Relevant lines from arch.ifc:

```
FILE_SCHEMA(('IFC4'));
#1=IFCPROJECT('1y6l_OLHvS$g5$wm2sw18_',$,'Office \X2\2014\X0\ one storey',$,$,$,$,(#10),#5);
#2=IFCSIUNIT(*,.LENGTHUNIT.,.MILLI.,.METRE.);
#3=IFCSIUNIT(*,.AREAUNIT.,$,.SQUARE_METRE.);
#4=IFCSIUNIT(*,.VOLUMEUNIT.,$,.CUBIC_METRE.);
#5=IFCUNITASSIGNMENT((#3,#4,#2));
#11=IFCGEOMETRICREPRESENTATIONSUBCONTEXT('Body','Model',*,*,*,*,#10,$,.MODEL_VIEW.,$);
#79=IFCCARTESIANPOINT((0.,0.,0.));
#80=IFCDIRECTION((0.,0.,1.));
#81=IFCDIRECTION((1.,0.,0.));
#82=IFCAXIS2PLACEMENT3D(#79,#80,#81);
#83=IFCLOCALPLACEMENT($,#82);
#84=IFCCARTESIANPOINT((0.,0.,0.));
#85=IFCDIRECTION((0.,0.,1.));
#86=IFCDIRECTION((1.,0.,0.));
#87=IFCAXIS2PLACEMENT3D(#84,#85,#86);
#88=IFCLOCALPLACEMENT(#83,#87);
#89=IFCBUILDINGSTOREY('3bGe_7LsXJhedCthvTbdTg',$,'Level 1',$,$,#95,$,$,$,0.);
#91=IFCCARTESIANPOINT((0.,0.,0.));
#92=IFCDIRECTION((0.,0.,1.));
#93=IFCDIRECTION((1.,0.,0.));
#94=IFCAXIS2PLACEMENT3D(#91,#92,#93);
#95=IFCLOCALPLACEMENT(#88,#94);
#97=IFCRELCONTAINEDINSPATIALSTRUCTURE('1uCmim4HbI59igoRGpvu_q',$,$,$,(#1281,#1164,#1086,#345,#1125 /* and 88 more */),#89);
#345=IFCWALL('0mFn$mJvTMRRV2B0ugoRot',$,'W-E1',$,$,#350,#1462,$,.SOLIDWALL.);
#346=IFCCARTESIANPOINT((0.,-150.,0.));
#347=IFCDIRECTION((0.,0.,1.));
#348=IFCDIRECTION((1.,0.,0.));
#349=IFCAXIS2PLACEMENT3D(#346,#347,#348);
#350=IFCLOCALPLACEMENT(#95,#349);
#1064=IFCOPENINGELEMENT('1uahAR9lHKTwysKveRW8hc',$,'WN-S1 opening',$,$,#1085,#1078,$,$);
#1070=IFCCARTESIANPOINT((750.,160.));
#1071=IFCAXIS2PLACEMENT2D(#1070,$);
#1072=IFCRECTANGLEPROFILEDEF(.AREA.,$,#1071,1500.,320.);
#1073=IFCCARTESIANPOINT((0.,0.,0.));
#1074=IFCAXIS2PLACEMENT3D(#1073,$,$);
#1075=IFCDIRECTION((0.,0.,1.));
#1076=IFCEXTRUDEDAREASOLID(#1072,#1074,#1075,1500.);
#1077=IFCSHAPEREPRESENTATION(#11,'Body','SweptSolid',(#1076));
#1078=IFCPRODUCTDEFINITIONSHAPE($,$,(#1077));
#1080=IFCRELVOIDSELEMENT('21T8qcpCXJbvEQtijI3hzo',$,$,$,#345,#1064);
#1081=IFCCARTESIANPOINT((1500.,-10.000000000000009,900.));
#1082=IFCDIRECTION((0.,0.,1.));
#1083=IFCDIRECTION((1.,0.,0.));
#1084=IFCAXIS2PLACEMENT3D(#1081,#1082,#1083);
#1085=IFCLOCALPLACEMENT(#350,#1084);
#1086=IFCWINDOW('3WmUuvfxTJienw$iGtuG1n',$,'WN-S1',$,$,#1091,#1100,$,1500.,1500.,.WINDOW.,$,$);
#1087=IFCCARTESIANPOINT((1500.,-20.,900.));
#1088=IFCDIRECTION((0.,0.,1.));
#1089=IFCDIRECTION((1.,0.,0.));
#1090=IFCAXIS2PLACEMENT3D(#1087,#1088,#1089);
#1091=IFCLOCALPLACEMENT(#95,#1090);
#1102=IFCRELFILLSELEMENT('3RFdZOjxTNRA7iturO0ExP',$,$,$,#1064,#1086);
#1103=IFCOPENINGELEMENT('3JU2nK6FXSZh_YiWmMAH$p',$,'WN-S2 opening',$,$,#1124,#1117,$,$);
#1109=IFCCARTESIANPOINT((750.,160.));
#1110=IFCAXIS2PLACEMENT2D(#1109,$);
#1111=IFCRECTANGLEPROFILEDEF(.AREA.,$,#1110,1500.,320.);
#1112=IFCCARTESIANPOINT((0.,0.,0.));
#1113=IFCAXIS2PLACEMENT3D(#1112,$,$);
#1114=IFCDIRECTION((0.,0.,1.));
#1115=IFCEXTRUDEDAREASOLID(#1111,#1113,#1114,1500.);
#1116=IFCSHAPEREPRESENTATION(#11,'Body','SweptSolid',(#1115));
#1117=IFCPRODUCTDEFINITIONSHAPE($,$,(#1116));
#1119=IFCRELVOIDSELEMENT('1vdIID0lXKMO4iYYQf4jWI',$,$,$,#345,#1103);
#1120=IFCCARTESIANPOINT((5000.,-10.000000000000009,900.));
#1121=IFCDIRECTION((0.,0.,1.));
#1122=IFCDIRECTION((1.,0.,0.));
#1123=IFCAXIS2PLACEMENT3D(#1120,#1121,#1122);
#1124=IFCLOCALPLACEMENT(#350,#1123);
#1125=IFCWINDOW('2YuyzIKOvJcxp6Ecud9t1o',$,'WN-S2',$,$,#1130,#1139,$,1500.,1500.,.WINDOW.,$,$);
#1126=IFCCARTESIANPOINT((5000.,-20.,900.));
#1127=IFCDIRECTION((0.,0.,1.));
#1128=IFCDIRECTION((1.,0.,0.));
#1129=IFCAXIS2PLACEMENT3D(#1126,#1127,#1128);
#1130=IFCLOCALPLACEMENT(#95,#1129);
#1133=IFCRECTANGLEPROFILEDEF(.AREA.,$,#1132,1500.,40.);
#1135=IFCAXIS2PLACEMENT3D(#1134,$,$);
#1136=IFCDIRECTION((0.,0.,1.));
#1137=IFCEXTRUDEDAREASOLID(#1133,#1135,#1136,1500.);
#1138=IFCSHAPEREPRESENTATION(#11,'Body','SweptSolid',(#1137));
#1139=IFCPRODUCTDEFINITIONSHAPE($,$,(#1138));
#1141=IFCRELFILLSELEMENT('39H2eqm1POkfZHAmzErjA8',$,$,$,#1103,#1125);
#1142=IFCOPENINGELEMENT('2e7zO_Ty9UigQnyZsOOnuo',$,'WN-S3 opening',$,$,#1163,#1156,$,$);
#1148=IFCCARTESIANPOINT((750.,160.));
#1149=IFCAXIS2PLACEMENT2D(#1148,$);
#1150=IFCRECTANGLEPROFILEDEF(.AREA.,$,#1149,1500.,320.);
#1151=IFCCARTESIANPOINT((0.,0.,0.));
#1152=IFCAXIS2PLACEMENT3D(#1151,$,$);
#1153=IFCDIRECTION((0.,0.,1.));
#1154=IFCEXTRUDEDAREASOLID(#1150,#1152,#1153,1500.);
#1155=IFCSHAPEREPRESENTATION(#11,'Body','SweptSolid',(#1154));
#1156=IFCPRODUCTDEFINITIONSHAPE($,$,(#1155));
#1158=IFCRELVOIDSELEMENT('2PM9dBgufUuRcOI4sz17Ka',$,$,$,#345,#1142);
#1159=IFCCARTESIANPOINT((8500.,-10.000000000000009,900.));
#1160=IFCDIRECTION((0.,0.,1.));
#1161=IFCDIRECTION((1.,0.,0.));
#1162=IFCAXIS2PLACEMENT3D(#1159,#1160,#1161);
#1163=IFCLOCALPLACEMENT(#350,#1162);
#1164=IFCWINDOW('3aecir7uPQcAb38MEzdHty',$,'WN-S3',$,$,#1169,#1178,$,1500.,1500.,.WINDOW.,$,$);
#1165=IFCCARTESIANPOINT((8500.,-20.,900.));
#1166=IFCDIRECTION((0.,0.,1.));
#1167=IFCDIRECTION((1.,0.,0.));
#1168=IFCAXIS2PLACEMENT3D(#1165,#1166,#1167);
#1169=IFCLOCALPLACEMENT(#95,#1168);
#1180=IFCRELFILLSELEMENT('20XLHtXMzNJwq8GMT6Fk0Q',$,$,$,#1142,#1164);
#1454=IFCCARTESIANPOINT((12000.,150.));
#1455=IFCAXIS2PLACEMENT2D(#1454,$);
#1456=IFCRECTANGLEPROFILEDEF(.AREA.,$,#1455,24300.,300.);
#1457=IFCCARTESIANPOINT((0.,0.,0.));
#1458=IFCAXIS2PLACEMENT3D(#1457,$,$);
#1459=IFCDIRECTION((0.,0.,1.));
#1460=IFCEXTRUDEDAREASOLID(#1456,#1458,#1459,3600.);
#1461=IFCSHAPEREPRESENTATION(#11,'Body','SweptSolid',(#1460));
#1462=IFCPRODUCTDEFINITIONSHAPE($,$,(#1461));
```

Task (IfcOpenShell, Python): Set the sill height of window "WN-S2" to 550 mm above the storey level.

```python
import numpy as np
import ifcopenshell
import ifcopenshell.api.geometry
import ifcopenshell.geom
import ifcopenshell.util.element
import ifcopenshell.util.placement
import ifcopenshell.util.shape
import ifcopenshell.util.unit

model = ifcopenshell.open("arch.ifc")
unit_scale = ifcopenshell.util.unit.calculate_unit_scale(model)

window = model.by_guid("2YuyzIKOvJcxp6Ecud9t1o")
opening = window.FillsVoids[0].RelatingOpeningElement
storey = ifcopenshell.util.element.get_container(window, ifc_class="IfcBuildingStorey")
level = ifcopenshell.util.placement.get_local_placement(storey.ObjectPlacement)[2, 3]

# The opening's origin need not be at the sill, so measure its lowest point.
shape = ifcopenshell.geom.create_shape(ifcopenshell.geom.settings(), opening)
bottom = ifcopenshell.util.shape.get_shape_bottom_elevation(shape, shape.geometry) / unit_scale
dz = level + 0.55 / unit_scale - bottom

shift = np.array([0.0, 0.0, dz])
# The window is not placed relative to its opening, so move both.
for product in (opening, window):
    matrix = ifcopenshell.util.placement.get_local_placement(product.ObjectPlacement)
    matrix[:3, 3] += shift
    ifcopenshell.api.geometry.edit_object_placement(model, product=product, matrix=matrix, is_si=False)

print(f"moved by {dz * unit_scale:+.3f} m")

model.write("arch_rev.ifc")
```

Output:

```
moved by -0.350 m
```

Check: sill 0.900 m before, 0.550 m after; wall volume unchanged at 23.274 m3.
